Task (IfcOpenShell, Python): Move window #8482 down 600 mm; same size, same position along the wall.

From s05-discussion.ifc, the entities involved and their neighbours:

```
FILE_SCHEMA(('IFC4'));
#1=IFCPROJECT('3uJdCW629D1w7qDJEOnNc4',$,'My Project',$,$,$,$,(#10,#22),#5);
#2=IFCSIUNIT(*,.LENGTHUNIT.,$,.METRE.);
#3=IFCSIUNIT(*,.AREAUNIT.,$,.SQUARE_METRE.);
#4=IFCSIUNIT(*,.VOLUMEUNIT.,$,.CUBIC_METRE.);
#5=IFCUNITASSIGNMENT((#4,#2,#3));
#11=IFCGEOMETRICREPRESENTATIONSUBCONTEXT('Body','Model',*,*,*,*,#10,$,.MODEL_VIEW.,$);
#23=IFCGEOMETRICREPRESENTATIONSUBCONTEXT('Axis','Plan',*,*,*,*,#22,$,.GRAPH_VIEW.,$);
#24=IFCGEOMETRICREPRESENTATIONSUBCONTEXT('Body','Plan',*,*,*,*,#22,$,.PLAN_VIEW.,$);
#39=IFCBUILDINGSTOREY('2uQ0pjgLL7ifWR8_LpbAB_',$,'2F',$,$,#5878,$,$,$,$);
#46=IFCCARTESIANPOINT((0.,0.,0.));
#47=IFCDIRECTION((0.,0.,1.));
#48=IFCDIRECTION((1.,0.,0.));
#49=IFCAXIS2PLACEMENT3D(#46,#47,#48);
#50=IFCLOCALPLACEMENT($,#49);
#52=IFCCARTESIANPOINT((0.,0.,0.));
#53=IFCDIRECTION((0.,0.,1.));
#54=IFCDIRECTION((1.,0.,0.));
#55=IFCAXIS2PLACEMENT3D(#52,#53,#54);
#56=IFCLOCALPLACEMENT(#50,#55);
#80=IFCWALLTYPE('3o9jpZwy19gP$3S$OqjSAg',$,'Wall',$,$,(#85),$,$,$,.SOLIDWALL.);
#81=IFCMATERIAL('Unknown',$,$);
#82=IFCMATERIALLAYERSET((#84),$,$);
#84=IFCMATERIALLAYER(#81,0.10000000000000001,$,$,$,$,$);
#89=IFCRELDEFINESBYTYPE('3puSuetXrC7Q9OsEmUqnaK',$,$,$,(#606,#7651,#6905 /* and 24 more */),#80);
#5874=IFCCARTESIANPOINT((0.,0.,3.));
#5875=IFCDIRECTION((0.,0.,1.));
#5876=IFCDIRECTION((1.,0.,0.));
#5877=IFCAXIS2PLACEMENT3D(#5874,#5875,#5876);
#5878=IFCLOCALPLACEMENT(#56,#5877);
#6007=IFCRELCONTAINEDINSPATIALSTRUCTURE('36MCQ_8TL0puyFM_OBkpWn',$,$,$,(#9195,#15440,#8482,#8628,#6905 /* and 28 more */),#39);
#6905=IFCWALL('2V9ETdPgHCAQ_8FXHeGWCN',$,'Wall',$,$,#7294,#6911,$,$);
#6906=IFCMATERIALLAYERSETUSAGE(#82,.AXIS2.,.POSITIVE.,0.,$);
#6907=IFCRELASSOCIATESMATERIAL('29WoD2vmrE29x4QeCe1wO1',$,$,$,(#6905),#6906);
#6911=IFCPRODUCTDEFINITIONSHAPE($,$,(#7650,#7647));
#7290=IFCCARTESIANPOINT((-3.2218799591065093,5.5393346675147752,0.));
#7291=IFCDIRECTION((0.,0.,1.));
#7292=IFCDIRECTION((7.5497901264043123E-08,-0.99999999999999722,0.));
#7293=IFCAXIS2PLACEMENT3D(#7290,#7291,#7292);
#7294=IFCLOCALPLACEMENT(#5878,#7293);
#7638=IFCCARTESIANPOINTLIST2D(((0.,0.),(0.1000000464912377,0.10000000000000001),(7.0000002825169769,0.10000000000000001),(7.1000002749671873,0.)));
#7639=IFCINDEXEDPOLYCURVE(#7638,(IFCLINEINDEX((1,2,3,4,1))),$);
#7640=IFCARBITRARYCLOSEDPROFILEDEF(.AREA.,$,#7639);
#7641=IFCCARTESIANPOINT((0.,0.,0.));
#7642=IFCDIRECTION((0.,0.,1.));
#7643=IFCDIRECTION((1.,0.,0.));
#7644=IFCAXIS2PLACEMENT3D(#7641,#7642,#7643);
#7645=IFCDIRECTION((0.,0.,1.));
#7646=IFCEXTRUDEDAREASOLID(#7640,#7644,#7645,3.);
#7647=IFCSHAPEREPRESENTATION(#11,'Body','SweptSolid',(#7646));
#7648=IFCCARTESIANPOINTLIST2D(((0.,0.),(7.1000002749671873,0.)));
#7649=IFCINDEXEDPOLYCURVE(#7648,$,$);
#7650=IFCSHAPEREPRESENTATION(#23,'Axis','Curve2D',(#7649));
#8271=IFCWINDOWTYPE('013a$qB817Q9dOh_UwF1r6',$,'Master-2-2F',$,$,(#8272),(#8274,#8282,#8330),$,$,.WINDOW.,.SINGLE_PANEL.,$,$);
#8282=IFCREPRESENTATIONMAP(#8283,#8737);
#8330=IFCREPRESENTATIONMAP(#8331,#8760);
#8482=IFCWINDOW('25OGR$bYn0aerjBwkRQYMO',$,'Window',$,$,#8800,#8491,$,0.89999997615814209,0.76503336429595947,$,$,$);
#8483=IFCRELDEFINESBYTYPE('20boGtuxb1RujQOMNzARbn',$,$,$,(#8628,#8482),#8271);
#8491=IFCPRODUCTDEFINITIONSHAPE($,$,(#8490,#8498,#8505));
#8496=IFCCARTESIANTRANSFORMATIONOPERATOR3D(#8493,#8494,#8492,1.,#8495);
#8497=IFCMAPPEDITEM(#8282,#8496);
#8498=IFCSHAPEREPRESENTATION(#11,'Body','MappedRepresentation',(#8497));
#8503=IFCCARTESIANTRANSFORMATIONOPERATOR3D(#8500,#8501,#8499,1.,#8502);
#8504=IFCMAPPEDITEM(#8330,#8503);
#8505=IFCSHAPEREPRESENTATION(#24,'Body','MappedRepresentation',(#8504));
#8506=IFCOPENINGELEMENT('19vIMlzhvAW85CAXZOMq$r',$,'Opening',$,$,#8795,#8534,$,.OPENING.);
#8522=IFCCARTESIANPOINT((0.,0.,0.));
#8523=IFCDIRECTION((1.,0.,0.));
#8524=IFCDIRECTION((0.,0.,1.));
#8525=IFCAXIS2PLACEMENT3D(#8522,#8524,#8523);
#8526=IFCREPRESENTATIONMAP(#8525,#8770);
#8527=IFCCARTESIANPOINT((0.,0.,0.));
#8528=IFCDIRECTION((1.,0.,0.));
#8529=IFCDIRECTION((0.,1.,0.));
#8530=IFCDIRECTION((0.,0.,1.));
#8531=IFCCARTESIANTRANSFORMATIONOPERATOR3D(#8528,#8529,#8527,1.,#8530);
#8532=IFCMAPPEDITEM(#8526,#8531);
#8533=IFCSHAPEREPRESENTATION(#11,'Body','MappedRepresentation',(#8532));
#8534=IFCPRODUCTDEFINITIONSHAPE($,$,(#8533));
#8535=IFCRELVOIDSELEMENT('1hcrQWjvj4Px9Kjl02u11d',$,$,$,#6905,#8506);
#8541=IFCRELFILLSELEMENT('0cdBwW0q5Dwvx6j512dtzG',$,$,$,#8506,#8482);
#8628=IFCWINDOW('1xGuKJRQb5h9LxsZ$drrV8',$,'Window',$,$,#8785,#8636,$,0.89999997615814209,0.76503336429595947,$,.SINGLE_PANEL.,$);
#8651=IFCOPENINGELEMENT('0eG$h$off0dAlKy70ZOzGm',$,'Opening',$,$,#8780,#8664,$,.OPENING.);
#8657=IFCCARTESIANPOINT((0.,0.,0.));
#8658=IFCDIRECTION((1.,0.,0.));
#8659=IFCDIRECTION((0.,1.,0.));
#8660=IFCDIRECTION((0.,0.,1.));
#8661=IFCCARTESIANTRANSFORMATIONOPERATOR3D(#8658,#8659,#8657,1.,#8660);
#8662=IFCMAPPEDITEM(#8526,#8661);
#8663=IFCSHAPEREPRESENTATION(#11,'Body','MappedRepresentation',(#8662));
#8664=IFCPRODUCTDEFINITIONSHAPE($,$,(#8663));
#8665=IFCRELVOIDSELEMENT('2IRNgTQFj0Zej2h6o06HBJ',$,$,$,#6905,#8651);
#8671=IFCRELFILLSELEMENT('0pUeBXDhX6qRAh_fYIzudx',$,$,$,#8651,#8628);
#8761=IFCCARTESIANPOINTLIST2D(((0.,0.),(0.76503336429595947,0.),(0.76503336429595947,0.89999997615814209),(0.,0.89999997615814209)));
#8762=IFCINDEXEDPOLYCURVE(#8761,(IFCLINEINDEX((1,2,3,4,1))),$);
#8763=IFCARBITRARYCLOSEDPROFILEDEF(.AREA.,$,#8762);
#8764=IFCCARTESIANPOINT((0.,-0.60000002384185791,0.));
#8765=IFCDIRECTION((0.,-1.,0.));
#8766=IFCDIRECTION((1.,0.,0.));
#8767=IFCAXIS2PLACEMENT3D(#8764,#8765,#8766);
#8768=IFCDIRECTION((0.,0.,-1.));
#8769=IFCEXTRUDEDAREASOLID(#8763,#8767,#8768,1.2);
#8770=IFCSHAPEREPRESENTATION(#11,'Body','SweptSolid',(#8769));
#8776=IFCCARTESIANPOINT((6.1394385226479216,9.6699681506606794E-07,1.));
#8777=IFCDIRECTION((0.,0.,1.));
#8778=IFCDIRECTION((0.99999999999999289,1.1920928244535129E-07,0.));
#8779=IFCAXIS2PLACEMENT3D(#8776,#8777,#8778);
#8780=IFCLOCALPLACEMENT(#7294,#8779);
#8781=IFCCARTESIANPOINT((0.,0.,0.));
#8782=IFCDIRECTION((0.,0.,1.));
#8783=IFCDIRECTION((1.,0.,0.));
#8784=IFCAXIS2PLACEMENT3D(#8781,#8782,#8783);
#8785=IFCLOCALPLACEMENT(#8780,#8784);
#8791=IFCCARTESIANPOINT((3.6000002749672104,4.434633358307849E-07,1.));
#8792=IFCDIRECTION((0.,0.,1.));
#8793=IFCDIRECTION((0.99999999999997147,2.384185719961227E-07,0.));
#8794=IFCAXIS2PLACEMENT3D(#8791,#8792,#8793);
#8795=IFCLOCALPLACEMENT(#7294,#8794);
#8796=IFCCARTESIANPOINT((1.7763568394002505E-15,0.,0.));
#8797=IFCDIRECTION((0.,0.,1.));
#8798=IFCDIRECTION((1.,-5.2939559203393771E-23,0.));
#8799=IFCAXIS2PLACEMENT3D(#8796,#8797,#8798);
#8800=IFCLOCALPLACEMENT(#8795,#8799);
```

```python
import numpy as np
import ifcopenshell
import ifcopenshell.api.geometry
import ifcopenshell.util.placement
import ifcopenshell.util.unit

model = ifcopenshell.open("s05-discussion.ifc")
unit_scale = ifcopenshell.util.unit.calculate_unit_scale(model)

window = model.by_id(8482)
opening = window.FillsVoids[0].RelatingOpeningElement
dz = -0.6 / unit_scale

shift = np.array([0.0, 0.0, dz])
# The window is placed relative to its opening, so it follows when the opening moves.
matrix = ifcopenshell.util.placement.get_local_placement(opening.ObjectPlacement)
matrix[:3, 3] += shift
ifcopenshell.api.geometry.edit_object_placement(
    model, product=opening, matrix=matrix, is_si=False, should_transform_children=True
)

print(f"moved by {dz * unit_scale:+.3f} m")

model.write("s05-discussion_edited.ifc")
```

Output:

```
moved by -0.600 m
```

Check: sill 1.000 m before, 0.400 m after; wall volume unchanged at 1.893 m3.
